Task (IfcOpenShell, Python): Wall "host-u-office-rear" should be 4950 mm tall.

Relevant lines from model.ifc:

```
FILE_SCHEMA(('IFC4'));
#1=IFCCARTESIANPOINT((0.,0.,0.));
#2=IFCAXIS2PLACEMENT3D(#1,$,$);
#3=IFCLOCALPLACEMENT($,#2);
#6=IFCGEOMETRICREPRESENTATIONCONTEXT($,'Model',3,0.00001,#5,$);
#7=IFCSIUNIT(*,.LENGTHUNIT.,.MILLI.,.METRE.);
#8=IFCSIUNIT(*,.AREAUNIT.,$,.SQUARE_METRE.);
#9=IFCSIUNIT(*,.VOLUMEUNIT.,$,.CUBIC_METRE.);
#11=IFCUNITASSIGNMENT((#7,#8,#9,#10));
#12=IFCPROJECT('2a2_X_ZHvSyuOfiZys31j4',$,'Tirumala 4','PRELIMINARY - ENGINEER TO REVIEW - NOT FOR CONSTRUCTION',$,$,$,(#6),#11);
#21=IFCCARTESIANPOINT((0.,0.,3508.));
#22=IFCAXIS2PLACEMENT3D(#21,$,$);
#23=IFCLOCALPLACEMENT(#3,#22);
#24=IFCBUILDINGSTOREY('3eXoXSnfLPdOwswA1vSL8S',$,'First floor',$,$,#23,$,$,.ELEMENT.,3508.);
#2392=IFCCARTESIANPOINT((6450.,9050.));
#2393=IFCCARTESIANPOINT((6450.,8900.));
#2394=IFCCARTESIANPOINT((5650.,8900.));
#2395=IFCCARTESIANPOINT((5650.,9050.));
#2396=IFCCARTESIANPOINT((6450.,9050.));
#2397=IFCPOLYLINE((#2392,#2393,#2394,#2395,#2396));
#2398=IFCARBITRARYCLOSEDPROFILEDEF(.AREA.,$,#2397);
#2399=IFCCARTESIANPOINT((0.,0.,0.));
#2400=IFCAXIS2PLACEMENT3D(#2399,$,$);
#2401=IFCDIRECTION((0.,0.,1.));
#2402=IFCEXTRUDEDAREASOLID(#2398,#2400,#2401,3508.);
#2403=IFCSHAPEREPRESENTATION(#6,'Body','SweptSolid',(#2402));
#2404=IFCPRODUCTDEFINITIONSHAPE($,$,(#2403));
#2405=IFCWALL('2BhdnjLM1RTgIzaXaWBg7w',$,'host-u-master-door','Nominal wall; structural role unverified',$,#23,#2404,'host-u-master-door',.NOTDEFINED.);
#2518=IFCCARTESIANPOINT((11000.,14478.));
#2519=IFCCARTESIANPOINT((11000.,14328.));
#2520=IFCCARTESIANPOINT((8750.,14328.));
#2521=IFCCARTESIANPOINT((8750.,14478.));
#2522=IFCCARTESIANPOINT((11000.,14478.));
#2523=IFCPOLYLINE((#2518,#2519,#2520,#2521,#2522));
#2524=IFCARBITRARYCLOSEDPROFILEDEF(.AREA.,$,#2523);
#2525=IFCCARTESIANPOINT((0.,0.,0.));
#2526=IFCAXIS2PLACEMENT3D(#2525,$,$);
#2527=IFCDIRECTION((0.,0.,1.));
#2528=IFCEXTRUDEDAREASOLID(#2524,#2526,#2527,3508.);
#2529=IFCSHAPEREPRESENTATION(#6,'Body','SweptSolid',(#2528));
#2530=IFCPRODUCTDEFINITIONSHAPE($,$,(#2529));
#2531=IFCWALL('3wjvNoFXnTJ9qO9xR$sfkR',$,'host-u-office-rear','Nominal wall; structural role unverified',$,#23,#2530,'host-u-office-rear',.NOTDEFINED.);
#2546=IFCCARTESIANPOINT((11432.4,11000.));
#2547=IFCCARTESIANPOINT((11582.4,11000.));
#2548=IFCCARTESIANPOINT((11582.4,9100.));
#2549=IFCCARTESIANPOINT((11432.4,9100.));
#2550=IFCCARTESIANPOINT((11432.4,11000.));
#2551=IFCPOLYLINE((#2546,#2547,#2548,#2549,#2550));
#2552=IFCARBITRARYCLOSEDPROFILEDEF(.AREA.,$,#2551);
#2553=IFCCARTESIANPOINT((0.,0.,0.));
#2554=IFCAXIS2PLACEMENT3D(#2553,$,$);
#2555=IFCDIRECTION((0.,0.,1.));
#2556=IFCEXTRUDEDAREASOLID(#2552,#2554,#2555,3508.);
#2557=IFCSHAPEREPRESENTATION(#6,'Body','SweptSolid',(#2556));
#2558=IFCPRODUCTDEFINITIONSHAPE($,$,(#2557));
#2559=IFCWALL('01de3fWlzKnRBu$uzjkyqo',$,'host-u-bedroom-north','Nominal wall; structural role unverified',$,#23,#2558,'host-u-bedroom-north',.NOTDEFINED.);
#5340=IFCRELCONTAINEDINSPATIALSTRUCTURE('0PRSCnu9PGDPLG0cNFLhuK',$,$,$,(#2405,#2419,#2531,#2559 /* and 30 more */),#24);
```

```python
import ifcopenshell
import ifcopenshell.geom
import ifcopenshell.util.shape
import ifcopenshell.util.unit

model = ifcopenshell.open("model.ifc")
unit_scale = ifcopenshell.util.unit.calculate_unit_scale(model)
settings = ifcopenshell.geom.settings()


def volume(element):
    """Net volume in cubic metres, openings subtracted."""
    shape = ifcopenshell.geom.create_shape(settings, element)
    return ifcopenshell.util.shape.get_volume(shape.geometry)


wall = model.by_id(2531)
before = volume(wall)

body = next(r for r in wall.Representation.Representations if r.RepresentationIdentifier == "Body")
solid = body.Items[0]
old_height = solid.Depth
solid.Depth = 4.95 / unit_scale
after = volume(wall)

print(f"height {old_height:g} -> {solid.Depth:g}, volume {before:.3f} -> {after:.3f} m3")

model.write("model_v2.ifc")
```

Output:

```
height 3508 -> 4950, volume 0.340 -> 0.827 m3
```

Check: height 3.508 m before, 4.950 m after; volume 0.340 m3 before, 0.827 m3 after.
